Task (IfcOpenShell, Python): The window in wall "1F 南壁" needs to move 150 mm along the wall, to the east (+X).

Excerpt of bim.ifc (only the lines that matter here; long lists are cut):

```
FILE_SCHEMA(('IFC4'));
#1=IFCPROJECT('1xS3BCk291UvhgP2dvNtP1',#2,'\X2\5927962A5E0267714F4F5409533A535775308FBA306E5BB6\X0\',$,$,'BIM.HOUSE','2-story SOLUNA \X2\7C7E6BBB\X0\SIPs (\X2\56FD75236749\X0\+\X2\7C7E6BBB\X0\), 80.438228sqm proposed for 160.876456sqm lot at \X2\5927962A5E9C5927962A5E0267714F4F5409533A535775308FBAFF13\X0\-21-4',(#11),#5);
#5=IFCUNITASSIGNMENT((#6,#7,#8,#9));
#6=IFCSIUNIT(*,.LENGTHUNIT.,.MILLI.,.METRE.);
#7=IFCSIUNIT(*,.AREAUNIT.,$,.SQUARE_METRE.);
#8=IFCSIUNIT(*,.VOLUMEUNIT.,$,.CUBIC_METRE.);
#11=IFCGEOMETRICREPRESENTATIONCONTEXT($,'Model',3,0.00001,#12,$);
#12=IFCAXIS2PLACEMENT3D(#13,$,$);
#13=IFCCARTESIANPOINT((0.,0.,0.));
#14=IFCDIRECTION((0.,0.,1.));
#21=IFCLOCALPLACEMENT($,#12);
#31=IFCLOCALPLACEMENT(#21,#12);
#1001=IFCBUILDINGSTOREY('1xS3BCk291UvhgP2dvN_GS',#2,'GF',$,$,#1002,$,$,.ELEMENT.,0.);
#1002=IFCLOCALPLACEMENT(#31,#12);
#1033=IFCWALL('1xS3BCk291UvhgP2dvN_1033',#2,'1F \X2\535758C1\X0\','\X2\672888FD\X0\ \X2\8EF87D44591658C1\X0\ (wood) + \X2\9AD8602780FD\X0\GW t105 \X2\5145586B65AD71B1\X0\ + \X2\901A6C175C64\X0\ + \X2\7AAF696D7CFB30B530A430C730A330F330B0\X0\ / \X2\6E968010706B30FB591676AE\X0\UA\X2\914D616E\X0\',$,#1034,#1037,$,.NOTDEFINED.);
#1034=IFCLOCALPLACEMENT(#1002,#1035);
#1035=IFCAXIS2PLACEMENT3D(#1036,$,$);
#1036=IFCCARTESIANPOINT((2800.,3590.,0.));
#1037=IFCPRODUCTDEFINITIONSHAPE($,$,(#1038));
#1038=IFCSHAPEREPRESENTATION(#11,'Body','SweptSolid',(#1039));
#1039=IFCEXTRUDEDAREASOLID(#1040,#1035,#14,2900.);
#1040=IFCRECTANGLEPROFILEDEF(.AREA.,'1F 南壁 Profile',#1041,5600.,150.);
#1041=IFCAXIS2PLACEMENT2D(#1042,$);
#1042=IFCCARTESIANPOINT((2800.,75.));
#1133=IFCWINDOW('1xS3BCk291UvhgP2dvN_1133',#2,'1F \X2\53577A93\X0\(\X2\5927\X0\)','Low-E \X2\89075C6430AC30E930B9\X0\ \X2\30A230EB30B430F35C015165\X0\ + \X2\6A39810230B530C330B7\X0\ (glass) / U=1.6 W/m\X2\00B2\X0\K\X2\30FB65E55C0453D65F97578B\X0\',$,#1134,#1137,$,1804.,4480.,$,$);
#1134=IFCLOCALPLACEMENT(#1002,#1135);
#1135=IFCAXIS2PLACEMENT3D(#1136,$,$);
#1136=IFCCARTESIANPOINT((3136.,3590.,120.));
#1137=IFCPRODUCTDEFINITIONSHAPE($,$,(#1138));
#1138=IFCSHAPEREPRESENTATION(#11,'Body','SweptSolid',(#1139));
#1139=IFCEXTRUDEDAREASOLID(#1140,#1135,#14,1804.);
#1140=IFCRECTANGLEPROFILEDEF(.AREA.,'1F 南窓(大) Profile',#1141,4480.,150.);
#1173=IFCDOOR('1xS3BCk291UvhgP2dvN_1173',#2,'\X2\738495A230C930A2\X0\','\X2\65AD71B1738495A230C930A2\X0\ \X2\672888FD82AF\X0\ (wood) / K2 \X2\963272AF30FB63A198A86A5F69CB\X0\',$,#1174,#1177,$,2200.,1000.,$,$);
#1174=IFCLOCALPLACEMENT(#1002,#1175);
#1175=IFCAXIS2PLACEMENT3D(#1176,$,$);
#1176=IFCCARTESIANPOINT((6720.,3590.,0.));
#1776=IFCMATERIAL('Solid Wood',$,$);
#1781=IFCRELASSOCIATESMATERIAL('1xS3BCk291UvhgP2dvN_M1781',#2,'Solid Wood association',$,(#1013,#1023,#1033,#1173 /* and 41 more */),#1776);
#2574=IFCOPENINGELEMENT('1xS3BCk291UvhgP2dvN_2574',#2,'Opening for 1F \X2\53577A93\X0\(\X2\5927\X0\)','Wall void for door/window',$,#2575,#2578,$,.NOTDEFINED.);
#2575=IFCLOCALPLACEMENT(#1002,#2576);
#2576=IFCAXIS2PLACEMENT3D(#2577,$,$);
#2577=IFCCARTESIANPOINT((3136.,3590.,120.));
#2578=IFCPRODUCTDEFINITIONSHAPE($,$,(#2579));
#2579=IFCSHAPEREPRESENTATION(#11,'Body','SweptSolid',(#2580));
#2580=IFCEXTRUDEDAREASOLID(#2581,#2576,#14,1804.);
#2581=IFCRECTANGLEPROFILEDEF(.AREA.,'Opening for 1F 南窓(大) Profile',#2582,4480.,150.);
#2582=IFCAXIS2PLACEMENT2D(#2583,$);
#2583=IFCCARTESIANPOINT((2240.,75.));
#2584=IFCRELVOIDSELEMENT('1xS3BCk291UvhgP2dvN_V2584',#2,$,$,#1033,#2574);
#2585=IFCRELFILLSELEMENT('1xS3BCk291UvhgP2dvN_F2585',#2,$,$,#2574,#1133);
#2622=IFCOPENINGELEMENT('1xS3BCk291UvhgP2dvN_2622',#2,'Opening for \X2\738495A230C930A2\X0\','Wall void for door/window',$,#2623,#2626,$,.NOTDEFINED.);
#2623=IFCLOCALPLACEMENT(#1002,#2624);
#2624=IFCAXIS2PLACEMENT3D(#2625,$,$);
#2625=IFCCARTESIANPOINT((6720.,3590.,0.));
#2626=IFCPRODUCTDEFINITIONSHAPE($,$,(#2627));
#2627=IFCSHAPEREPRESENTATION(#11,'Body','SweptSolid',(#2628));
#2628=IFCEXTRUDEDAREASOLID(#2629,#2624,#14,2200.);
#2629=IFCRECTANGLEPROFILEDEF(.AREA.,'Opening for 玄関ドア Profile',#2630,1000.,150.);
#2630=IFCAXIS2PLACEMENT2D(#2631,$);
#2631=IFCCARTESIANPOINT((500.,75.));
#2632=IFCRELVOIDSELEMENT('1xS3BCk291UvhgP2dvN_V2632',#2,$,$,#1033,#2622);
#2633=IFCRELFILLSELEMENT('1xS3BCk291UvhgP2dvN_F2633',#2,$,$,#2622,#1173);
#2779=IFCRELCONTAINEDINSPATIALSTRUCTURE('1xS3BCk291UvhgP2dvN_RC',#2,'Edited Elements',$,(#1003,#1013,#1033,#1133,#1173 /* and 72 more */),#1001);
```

```python
import ifcopenshell
import ifcopenshell.api.geometry
import ifcopenshell.util.placement
import ifcopenshell.util.unit

model = ifcopenshell.open("bim.ifc")
unit_scale = ifcopenshell.util.unit.calculate_unit_scale(model)

window = model.by_guid("1xS3BCk291UvhgP2dvN_1133")
opening = window.FillsVoids[0].RelatingOpeningElement
wall = opening.VoidsElements[0].RelatingBuildingElement

wall_matrix = ifcopenshell.util.placement.get_local_placement(wall.ObjectPlacement)
shift = wall_matrix[:3, 0] * 0.15 / unit_scale
before = ifcopenshell.util.placement.get_local_placement(window.ObjectPlacement)[:3, 3].copy()

# The window is not placed relative to its opening, so move both.
for product in (opening, window):
    matrix = ifcopenshell.util.placement.get_local_placement(product.ObjectPlacement)
    matrix[:3, 3] += shift
    ifcopenshell.api.geometry.edit_object_placement(model, product=product, matrix=matrix, is_si=False)

after = ifcopenshell.util.placement.get_local_placement(window.ObjectPlacement)[:3, 3]
print("window moved by", (after - before).round(3) + 0.0)

model.write("bim-out.ifc")
```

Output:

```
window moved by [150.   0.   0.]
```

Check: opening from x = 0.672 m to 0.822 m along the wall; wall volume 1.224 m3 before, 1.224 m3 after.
